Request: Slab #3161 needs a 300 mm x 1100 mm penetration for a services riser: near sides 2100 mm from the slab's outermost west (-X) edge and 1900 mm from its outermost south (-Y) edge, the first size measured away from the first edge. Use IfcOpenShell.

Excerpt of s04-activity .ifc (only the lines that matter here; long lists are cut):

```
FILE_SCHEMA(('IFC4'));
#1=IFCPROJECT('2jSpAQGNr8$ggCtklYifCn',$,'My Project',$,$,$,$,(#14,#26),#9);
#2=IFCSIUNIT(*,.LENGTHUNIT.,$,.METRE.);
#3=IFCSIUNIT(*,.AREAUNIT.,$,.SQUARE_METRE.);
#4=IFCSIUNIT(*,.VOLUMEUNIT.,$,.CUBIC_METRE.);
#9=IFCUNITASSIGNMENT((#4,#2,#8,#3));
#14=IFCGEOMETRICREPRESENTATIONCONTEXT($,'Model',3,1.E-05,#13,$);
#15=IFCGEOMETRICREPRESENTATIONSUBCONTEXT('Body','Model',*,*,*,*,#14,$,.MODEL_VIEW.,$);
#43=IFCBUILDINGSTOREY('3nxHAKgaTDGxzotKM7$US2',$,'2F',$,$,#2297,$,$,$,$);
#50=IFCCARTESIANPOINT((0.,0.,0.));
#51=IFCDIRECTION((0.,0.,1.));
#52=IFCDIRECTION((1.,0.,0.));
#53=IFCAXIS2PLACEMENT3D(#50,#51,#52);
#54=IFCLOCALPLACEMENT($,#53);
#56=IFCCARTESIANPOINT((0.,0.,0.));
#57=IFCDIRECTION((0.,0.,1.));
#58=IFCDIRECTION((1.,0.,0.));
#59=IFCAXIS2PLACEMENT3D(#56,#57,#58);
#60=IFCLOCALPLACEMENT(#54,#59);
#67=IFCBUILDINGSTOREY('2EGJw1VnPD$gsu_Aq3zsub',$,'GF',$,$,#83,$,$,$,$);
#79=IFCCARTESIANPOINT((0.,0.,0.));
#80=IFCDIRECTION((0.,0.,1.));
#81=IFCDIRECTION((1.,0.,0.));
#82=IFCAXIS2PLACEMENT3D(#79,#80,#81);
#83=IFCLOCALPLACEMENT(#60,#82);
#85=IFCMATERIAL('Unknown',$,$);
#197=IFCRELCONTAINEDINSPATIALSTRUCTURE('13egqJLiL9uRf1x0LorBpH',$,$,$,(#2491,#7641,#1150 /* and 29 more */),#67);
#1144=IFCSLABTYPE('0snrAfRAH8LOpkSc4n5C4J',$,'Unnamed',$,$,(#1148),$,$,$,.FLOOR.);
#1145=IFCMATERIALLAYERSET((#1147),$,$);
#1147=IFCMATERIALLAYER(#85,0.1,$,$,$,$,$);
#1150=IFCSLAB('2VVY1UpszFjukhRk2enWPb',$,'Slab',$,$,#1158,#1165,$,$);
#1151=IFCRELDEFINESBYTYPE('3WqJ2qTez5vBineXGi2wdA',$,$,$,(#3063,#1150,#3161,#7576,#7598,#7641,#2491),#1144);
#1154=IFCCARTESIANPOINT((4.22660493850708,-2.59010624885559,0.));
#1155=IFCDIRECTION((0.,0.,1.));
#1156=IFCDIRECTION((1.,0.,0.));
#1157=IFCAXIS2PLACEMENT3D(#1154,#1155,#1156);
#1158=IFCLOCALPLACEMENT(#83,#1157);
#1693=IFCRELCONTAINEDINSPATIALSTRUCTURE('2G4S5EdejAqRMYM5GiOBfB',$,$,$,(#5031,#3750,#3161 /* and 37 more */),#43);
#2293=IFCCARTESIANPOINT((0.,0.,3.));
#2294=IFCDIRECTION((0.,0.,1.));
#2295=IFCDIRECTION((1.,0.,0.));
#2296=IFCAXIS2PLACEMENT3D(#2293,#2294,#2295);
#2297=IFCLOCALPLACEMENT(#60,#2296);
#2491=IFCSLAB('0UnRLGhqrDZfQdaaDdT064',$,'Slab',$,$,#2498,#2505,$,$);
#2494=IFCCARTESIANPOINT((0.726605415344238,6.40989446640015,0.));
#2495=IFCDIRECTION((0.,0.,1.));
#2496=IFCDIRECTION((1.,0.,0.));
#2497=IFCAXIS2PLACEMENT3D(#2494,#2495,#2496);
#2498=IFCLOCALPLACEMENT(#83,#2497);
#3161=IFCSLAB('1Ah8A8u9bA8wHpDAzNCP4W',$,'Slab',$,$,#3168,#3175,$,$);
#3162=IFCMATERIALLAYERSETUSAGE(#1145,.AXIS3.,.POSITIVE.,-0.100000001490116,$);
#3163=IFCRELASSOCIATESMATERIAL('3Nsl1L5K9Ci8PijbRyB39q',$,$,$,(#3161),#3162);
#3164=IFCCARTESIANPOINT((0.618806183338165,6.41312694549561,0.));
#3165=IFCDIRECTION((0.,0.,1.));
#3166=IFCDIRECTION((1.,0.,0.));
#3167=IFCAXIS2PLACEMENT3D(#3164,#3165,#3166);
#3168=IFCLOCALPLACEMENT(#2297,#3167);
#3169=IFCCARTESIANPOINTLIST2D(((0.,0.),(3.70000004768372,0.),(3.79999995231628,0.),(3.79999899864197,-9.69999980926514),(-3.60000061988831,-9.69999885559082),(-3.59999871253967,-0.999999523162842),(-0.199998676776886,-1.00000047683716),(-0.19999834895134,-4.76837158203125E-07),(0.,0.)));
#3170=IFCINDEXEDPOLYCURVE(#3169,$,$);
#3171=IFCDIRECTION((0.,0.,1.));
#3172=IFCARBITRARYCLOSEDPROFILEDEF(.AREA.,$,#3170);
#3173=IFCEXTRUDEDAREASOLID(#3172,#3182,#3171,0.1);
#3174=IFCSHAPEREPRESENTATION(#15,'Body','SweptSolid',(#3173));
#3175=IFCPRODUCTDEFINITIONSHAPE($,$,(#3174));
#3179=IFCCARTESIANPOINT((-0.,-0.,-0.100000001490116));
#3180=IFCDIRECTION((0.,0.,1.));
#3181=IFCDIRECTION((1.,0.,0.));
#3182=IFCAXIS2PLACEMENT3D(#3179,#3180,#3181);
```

```python
import numpy as np
import ifcopenshell
import ifcopenshell.api.feature
import ifcopenshell.api.geometry
import ifcopenshell.api.root
import ifcopenshell.geom
import ifcopenshell.util.placement
import ifcopenshell.util.representation
import ifcopenshell.util.shape
import ifcopenshell.util.unit

model = ifcopenshell.open("s04-activity .ifc")
unit_scale = ifcopenshell.util.unit.calculate_unit_scale(model)
settings = ifcopenshell.geom.settings()


def volume(element):
    """Net volume in cubic metres, openings subtracted."""
    shape = ifcopenshell.geom.create_shape(settings, element)
    return ifcopenshell.util.shape.get_volume(shape.geometry)


slab = model.by_guid("1Ah8A8u9bA8wHpDAzNCP4W")
before = volume(slab)

# Extent in the slab's own axes, in metres. The edges named are its -X and -Y sides.
slab_shape = ifcopenshell.geom.create_shape(settings, slab)
vertices = ifcopenshell.util.shape.get_vertices(slab_shape.geometry)
x_min, y_min, bottom = vertices.min(axis=0)
top = vertices[:, 2].max()

opening = ifcopenshell.api.root.create_entity(model, ifc_class="IfcOpeningElement", name="Services riser opening", predefined_type="OPENING")
context = ifcopenshell.util.representation.get_context(model, "Model", "Body", "MODEL_VIEW")
width, depth = 0.3, 1.1
outline = [(0.0, 0.0), (width, 0.0), (width, depth), (0.0, depth), (0.0, 0.0)]
# Overshoot both faces by 50 mm so the cut is clean.
shape = ifcopenshell.api.geometry.add_slab_representation(
    model, context=context, depth=top - bottom + 0.1, polyline=outline
)
ifcopenshell.api.geometry.assign_representation(model, product=opening, representation=shape)

matrix = ifcopenshell.util.placement.get_local_placement(slab.ObjectPlacement)
matrix[:, 3] = matrix @ np.append(np.array([x_min + 2.1, y_min + 1.9, bottom - 0.05]) / unit_scale, 1.0)
ifcopenshell.api.geometry.edit_object_placement(model, product=opening, matrix=matrix, is_si=False)
ifcopenshell.api.feature.add_feature(model, feature=opening, element=slab)

after = volume(slab)

print(f"slab volume {before:.3f} -> {after:.3f} m3")

model.write("s04-activity _v2.ifc")
```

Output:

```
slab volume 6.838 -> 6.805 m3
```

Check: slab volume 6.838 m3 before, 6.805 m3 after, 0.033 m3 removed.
